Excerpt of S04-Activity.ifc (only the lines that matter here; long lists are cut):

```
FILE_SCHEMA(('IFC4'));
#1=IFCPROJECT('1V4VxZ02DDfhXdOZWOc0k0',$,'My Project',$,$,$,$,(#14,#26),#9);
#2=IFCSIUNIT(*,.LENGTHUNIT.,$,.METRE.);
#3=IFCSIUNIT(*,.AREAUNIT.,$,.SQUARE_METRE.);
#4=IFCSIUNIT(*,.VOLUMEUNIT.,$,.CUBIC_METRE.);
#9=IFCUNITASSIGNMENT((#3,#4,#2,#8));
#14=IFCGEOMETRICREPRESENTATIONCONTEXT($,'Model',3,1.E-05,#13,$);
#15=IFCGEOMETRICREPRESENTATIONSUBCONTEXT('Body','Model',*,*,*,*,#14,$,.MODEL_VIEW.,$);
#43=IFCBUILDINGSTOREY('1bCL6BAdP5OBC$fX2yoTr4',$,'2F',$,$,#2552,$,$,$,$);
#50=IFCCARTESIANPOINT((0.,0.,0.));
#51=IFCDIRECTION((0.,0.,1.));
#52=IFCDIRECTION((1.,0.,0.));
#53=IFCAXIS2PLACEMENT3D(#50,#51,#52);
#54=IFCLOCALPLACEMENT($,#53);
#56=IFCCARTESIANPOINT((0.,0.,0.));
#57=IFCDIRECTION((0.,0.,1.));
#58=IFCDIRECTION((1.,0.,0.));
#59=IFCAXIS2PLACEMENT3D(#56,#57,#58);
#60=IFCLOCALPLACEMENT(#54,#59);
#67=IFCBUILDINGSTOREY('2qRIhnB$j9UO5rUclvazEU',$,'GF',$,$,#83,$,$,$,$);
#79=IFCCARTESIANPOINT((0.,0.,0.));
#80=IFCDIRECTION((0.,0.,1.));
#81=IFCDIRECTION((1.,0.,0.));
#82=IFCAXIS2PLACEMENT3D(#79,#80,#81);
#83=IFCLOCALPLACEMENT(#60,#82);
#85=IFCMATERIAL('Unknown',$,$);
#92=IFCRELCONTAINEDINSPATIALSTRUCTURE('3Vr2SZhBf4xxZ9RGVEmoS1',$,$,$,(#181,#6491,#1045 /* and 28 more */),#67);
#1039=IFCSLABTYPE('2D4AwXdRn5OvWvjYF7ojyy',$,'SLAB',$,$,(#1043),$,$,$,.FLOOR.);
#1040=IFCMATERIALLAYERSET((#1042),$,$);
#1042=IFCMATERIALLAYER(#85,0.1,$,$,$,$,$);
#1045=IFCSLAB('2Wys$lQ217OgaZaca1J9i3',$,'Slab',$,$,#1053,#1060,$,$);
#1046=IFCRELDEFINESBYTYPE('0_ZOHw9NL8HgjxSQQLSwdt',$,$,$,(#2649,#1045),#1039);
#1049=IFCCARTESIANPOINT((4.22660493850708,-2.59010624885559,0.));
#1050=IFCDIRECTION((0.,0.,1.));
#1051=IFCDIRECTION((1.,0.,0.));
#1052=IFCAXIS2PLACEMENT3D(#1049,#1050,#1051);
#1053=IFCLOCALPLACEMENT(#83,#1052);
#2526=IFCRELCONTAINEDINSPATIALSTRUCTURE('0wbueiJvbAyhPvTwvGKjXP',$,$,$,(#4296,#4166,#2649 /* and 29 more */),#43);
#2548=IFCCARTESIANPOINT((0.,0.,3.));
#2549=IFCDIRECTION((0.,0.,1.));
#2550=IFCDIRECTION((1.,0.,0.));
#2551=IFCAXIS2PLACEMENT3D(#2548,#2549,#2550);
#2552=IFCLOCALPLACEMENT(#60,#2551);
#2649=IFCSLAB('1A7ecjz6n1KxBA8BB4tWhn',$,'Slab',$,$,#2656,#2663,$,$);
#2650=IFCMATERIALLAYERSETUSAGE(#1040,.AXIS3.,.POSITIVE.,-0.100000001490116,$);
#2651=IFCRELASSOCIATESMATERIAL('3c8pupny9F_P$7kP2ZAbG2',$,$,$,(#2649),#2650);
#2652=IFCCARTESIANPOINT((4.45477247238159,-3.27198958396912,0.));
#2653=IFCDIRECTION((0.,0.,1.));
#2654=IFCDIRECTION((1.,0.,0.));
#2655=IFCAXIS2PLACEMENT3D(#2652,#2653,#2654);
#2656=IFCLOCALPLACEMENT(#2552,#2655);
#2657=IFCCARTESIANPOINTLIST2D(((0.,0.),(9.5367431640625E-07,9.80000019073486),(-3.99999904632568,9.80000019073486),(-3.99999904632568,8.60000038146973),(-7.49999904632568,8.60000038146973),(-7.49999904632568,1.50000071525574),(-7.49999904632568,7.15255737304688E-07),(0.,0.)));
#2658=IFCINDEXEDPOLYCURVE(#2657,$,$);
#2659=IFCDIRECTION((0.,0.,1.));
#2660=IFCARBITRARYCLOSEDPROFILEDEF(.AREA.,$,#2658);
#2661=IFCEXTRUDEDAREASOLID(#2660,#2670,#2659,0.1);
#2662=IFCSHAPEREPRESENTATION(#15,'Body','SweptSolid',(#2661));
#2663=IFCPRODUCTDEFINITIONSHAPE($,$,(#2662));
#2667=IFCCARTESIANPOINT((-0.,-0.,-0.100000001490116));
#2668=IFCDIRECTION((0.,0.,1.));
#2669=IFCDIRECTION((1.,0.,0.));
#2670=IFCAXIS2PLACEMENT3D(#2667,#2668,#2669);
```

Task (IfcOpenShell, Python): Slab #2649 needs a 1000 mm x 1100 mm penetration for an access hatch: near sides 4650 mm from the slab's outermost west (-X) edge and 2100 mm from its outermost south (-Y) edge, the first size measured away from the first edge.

```python
import numpy as np
import ifcopenshell
import ifcopenshell.api.feature
import ifcopenshell.api.geometry
import ifcopenshell.api.root
import ifcopenshell.geom
import ifcopenshell.util.placement
import ifcopenshell.util.representation
import ifcopenshell.util.shape
import ifcopenshell.util.unit

model = ifcopenshell.open("S04-Activity.ifc")
unit_scale = ifcopenshell.util.unit.calculate_unit_scale(model)
settings = ifcopenshell.geom.settings()


def volume(element):
    """Net volume in cubic metres, openings subtracted."""
    shape = ifcopenshell.geom.create_shape(settings, element)
    return ifcopenshell.util.shape.get_volume(shape.geometry)


slab = model.by_guid("1A7ecjz6n1KxBA8BB4tWhn")
before = volume(slab)

# Extent in the slab's own axes, in metres. The edges named are its -X and -Y sides.
slab_shape = ifcopenshell.geom.create_shape(settings, slab)
vertices = ifcopenshell.util.shape.get_vertices(slab_shape.geometry)
x_min, y_min, bottom = vertices.min(axis=0)
top = vertices[:, 2].max()

opening = ifcopenshell.api.root.create_entity(model, ifc_class="IfcOpeningElement", name="Access hatch opening", predefined_type="OPENING")
context = ifcopenshell.util.representation.get_context(model, "Model", "Body", "MODEL_VIEW")
width, depth = 1, 1.1
outline = [(0.0, 0.0), (width, 0.0), (width, depth), (0.0, depth), (0.0, 0.0)]
# Overshoot both faces by 50 mm so the cut is clean.
shape = ifcopenshell.api.geometry.add_slab_representation(
    model, context=context, depth=top - bottom + 0.1, polyline=outline
)
ifcopenshell.api.geometry.assign_representation(model, product=opening, representation=shape)

matrix = ifcopenshell.util.placement.get_local_placement(slab.ObjectPlacement)
matrix[:, 3] = matrix @ np.append(np.array([x_min + 4.65, y_min + 2.1, bottom - 0.05]) / unit_scale, 1.0)
ifcopenshell.api.geometry.edit_object_placement(model, product=opening, matrix=matrix, is_si=False)
ifcopenshell.api.feature.add_feature(model, feature=opening, element=slab)

after = volume(slab)

print(f"slab volume {before:.3f} -> {after:.3f} m3")

model.write("S04-Activity_edited.ifc")
```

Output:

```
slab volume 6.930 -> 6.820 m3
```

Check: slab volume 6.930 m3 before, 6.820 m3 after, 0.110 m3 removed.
